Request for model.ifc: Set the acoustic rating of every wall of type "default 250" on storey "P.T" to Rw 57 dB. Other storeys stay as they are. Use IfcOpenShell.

First a look at what the model holds.

```python
import ifcopenshell
import ifcopenshell.util.element

model = ifcopenshell.open("model.ifc")
print(model.schema)
storey = next(s for s in model.by_type("IfcBuildingStorey") if s.Name == "P.T")
walls = [e for e in ifcopenshell.util.element.get_decomposition(storey) if e.is_a("IfcWall")]
seen = {}
for e in walls:
    element_type = ifcopenshell.util.element.get_type(e)
    key = (element_type.Name if element_type != e and element_type else None, ifcopenshell.util.element.get_pset(e, "Pset_WallCommon", "AcousticRating"))
    seen[key] = seen.get(key, 0) + 1
for (name, value), count in sorted(seen.items(), key=str):
    print(count, "x", name, "|", value)
```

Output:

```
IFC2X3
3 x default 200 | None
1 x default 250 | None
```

```python
import ifcopenshell
import ifcopenshell.api.pset
import ifcopenshell.util.element

model = ifcopenshell.open("model.ifc")

storey = next(s for s in model.by_type("IfcBuildingStorey") if s.Name == "P.T")
walls = [e for e in ifcopenshell.util.element.get_decomposition(storey) if e.is_a("IfcWall")]

count = 0
for e in walls:
    element_type = ifcopenshell.util.element.get_type(e)
    if element_type in (None, e) or element_type.Name != "default 250":
        continue
    # add_pset returns the element's existing set when there is one.
    pset = ifcopenshell.api.pset.add_pset(model, product=e, name="Pset_WallCommon")
    ifcopenshell.api.pset.edit_pset(model, pset=pset, properties={"AcousticRating": "Rw 57 dB"})
    count += 1

print(count, "walls updated")

model.write("model_rev.ifc")
```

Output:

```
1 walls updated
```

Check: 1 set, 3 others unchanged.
